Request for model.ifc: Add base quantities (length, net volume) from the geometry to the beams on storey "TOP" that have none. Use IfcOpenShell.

First a look at what the model holds.

```python
import ifcopenshell
import ifcopenshell.util.element
import ifcopenshell.util.unit

model = ifcopenshell.open("model.ifc")
print(model.schema)
for unit_type in ("LENGTHUNIT", "AREAUNIT", "VOLUMEUNIT"):
    print(unit_type, ifcopenshell.util.unit.calculate_unit_scale(model, unit_type))
storey = next(s for s in model.by_type("IfcBuildingStorey") if s.Name == "TOP")
beams = [e for e in ifcopenshell.util.element.get_decomposition(storey) if e.is_a("IfcBeam")]
for e in sorted(beams, key=lambda e: e.id()):
    print(e.id(), e.is_a(), e.Name, list(ifcopenshell.util.element.get_psets(e, qtos_only=True)), sep=" | ")
```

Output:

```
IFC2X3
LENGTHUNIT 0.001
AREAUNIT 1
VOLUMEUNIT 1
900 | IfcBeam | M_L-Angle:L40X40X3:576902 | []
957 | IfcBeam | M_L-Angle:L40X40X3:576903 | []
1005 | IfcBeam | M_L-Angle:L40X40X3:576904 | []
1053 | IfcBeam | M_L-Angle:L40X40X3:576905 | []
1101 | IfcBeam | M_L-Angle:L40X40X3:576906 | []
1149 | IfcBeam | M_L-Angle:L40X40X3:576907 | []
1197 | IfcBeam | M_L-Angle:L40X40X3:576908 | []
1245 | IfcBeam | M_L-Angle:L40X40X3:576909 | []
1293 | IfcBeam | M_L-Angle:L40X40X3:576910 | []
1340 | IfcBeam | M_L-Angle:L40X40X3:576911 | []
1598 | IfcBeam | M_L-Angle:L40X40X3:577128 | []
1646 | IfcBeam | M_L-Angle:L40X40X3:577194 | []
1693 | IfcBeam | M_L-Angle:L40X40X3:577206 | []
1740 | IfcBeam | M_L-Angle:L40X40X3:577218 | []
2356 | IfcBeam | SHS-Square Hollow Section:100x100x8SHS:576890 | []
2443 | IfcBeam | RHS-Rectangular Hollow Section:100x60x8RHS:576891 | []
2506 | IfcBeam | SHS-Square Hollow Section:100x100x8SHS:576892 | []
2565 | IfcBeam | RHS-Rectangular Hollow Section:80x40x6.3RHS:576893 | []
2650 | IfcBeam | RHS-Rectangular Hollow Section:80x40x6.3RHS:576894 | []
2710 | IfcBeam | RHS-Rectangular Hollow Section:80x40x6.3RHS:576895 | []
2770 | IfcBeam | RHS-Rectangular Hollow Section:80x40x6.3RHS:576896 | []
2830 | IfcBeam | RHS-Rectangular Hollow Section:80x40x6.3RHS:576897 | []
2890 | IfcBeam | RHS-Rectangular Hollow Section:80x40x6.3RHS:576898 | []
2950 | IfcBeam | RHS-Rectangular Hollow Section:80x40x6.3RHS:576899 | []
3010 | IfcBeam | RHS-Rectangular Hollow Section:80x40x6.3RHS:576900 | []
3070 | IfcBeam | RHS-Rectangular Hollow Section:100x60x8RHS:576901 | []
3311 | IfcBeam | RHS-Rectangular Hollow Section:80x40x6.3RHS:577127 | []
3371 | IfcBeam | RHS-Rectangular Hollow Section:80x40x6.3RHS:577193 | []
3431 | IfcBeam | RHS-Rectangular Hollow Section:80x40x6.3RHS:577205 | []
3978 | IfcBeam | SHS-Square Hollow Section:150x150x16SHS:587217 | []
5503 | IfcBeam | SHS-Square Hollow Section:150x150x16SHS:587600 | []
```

```python
import ifcopenshell
import ifcopenshell.api.pset
import ifcopenshell.geom
import ifcopenshell.util.element
import ifcopenshell.util.shape
import ifcopenshell.util.unit

model = ifcopenshell.open("model.ifc")
unit_scale = ifcopenshell.util.unit.calculate_unit_scale(model)
volume_scale = ifcopenshell.util.unit.calculate_unit_scale(model, "VOLUMEUNIT")
settings = ifcopenshell.geom.settings()

storey = next(s for s in model.by_type("IfcBuildingStorey") if s.Name == "TOP")
beams = [e for e in ifcopenshell.util.element.get_decomposition(storey) if e.is_a("IfcBeam")]

for e in sorted(beams, key=lambda e: e.id()):
    if ifcopenshell.util.element.get_psets(e, qtos_only=True, should_inherit=False):
        continue
    # Geometry comes back in metres, in the element's own axes.
    shape = ifcopenshell.geom.create_shape(settings, e)
    values = {
        "Length": ifcopenshell.util.shape.get_max_xyz(shape.geometry) / unit_scale,
        "NetVolume": ifcopenshell.util.shape.get_volume(shape.geometry) / volume_scale,
    }
    qto = ifcopenshell.api.pset.add_qto(model, product=e, name="BaseQuantities")
    ifcopenshell.api.pset.edit_qto(model, qto=qto, properties=values)
    print(e.id(), {k: round(v, 3) for k, v in values.items()})

model.write("model_rev.ifc")
```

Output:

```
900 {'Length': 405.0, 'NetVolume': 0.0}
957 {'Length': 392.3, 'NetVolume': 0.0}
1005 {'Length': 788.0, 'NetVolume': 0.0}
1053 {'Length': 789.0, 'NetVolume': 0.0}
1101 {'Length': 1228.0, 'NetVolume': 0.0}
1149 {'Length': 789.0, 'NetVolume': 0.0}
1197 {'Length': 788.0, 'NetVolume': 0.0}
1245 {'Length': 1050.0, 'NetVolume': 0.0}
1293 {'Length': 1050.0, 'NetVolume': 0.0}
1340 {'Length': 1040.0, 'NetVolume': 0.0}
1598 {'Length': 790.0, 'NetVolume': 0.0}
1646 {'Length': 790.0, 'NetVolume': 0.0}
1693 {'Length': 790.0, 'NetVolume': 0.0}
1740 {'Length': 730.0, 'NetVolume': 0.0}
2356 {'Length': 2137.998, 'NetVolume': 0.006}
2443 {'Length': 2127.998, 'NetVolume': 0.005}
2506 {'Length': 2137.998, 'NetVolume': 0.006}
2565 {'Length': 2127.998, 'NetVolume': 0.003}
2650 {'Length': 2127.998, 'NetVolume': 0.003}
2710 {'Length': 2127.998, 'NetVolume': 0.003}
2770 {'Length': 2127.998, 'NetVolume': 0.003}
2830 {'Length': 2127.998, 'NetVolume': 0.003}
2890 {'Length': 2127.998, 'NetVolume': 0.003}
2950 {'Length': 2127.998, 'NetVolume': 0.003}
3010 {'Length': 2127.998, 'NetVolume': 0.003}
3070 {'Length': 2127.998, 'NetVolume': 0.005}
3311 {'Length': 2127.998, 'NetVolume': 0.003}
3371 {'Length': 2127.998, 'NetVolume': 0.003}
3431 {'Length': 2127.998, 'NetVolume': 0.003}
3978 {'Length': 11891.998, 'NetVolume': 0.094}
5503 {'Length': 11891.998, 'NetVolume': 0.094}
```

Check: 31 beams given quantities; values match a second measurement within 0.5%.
